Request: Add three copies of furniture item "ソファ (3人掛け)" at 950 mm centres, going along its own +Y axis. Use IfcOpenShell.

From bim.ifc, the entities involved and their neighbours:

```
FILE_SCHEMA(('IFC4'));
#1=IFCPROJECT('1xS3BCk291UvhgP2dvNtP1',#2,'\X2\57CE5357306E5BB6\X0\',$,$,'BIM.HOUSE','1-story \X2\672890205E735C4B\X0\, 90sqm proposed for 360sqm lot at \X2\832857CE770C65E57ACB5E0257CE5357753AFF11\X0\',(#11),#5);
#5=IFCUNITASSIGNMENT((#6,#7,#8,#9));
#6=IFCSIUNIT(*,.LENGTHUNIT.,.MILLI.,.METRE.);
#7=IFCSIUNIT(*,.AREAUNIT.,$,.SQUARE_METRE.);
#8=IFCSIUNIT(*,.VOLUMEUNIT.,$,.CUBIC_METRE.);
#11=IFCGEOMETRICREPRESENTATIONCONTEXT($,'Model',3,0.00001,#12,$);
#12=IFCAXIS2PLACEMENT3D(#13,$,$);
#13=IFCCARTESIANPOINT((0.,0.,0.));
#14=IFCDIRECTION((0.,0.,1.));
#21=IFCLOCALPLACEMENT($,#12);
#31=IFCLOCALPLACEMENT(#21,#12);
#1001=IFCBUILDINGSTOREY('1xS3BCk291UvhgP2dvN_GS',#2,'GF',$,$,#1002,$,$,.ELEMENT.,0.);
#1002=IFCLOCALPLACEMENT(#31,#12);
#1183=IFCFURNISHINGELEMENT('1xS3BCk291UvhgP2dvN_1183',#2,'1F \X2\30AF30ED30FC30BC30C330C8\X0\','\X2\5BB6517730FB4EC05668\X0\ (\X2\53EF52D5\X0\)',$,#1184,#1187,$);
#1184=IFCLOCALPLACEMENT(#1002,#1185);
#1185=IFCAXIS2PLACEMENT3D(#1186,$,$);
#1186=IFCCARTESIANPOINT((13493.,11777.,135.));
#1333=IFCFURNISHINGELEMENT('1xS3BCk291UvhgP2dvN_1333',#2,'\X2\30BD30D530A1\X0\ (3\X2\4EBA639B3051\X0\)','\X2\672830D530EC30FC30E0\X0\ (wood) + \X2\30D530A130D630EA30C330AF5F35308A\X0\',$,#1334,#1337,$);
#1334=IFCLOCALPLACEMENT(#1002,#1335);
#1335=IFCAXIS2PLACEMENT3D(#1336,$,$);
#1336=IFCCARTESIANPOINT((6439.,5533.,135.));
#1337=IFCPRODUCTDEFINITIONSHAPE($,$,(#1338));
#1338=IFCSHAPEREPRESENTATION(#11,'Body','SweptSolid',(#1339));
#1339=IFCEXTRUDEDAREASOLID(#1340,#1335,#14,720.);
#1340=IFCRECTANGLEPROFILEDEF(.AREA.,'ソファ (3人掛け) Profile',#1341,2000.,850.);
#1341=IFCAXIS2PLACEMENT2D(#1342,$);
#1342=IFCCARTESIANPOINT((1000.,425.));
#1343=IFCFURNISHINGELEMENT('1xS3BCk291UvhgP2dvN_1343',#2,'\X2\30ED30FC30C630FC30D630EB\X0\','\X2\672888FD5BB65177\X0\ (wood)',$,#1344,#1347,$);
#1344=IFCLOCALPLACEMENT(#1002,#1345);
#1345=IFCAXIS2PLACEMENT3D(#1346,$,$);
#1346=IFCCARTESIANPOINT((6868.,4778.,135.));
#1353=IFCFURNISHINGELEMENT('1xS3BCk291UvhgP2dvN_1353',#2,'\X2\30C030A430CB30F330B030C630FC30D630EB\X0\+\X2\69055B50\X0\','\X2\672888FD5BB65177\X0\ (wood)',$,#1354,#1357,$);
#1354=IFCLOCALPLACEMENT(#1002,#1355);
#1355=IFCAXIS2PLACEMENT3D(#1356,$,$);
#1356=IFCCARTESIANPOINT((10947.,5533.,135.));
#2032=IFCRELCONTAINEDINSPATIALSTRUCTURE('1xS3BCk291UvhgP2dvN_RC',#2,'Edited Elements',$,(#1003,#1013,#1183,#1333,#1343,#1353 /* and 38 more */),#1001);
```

```python
import ifcopenshell
import ifcopenshell.api.geometry
import ifcopenshell.api.root
import ifcopenshell.util.element
import ifcopenshell.util.placement
import ifcopenshell.util.unit

model = ifcopenshell.open("bim.ifc")
unit_scale = ifcopenshell.util.unit.calculate_unit_scale(model)


def reuse_history(source, copy):
    """copy_class also copies each property set's owner history, people and application; keep the originals."""
    for rel in copy.IsDefinedBy:
        if rel.is_a("IfcRelDefinesByProperties") and (history := rel.RelatingPropertyDefinition.OwnerHistory):
            rel.RelatingPropertyDefinition.OwnerHistory = source.OwnerHistory
            ifcopenshell.util.element.remove_deep2(model, history)


source = model.by_guid("1xS3BCk291UvhgP2dvN_1333")
base = ifcopenshell.util.placement.get_local_placement(source.ObjectPlacement)
step = base[:3, 1] * 0.95 / unit_scale

for i in range(1, 4):
    copy = ifcopenshell.api.root.copy_class(model, product=source)
    copy.Representation = ifcopenshell.util.element.copy_deep(
        model, source.Representation, exclude=["IfcGeometricRepresentationContext", "IfcRepresentationMap"]
    )
    reuse_history(source, copy)
    matrix = base.copy()
    matrix[:3, 3] += i * step
    print("added at", matrix[:3, 3].round(3) + 0.0)
    ifcopenshell.api.geometry.edit_object_placement(model, product=copy, matrix=matrix, is_si=False)

model.write("bim_edited.ifc")
```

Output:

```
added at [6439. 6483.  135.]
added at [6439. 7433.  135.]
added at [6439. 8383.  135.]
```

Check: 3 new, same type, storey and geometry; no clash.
